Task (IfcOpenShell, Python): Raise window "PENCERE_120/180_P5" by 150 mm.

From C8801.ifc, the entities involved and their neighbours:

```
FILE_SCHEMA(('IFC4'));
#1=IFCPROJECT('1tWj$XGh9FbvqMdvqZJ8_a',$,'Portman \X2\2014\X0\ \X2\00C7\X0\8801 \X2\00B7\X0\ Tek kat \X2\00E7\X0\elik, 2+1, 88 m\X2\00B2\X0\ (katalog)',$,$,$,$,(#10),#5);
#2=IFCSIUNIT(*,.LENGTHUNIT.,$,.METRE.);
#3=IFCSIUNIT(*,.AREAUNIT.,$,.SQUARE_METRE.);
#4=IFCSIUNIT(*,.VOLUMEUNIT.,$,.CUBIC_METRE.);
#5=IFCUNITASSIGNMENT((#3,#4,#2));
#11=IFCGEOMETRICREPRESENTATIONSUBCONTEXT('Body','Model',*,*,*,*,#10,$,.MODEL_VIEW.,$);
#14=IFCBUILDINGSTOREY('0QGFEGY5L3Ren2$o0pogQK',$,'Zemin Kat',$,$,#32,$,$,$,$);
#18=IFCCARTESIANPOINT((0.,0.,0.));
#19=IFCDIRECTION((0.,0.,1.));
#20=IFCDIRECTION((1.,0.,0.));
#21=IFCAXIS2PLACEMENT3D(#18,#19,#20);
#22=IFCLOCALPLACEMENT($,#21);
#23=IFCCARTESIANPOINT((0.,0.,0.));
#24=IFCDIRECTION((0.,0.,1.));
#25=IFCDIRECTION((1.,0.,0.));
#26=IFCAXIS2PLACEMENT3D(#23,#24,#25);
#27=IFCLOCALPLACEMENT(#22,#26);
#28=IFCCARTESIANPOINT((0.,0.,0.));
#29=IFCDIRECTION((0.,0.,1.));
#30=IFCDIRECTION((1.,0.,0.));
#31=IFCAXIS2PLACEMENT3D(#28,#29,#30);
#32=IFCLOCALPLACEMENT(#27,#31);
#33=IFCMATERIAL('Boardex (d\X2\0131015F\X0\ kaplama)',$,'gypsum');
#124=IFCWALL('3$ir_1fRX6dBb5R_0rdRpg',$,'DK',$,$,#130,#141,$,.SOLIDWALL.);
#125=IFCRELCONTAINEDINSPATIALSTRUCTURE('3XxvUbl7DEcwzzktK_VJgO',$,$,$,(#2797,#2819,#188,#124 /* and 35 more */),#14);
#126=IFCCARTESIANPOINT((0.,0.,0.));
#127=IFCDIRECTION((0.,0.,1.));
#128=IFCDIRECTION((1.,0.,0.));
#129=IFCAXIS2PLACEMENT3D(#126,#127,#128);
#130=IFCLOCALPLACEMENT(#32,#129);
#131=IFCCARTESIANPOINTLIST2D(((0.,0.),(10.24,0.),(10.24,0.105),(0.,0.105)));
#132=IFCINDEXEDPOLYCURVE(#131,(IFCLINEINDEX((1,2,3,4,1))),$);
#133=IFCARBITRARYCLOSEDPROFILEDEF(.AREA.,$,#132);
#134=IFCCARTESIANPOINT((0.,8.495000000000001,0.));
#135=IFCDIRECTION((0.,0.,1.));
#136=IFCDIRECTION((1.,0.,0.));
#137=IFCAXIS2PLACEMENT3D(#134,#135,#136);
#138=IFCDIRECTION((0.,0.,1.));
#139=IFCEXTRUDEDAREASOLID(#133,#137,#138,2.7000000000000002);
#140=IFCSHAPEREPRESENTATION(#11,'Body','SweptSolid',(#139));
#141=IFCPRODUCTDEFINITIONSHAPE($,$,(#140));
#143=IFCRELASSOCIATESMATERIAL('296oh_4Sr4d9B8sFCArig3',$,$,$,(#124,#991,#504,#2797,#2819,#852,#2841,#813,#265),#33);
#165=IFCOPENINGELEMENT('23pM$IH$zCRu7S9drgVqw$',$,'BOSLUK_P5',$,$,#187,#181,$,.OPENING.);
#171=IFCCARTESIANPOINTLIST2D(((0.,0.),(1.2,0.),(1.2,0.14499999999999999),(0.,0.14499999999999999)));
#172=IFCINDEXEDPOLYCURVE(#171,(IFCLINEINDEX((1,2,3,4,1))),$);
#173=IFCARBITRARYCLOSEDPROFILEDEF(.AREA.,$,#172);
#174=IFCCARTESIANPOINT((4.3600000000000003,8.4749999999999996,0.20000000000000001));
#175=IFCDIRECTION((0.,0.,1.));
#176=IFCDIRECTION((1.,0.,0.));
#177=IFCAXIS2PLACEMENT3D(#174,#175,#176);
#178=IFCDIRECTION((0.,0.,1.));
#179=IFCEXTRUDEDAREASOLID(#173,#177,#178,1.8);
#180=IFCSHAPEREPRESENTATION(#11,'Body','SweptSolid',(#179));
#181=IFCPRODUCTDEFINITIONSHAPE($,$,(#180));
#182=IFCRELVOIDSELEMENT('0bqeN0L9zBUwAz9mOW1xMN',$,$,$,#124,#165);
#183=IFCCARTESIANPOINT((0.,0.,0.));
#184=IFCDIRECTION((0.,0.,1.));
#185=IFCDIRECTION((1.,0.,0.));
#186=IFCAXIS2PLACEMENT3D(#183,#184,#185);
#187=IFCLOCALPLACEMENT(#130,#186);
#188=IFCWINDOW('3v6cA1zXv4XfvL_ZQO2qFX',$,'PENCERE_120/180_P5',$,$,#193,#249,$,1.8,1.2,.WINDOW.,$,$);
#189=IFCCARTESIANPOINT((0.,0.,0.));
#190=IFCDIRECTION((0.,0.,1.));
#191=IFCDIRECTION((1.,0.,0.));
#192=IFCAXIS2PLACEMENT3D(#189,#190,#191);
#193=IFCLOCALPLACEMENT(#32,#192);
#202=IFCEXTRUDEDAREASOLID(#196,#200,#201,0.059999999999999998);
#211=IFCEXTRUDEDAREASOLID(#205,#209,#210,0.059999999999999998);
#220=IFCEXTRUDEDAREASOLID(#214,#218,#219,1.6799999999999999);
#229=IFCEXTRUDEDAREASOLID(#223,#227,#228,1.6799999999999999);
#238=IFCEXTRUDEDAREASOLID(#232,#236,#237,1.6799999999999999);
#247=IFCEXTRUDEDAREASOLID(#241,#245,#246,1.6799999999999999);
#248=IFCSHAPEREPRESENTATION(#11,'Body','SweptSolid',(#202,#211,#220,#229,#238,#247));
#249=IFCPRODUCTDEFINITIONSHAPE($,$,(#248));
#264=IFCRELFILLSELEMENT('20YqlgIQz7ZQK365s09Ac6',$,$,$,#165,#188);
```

```python
import numpy as np
import ifcopenshell
import ifcopenshell.api.geometry
import ifcopenshell.util.placement
import ifcopenshell.util.unit

model = ifcopenshell.open("C8801.ifc")
unit_scale = ifcopenshell.util.unit.calculate_unit_scale(model)

window = model.by_id(188)
opening = window.FillsVoids[0].RelatingOpeningElement
dz = 0.15

shift = np.array([0.0, 0.0, dz])
# The window is not placed relative to its opening, so move both.
for product in (opening, window):
    matrix = ifcopenshell.util.placement.get_local_placement(product.ObjectPlacement)
    matrix[:3, 3] += shift
    ifcopenshell.api.geometry.edit_object_placement(model, product=product, matrix=matrix, is_si=False)

print(f"moved by {dz * unit_scale:+.3f} m")

model.write("C8801_v2.ifc")
```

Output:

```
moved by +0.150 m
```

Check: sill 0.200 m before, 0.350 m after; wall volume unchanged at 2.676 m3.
